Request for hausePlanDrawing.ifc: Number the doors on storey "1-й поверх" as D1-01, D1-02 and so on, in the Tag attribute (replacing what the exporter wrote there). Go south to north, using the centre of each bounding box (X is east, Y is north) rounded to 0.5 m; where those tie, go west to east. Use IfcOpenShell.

First a look at what the model holds.

```python
import ifcopenshell
import ifcopenshell.util.element
import ifcopenshell.util.placement

model = ifcopenshell.open("hausePlanDrawing.ifc")
print(model.schema)
storey = next(s for s in model.by_type("IfcBuildingStorey") if s.Name == "1-й поверх")
doors = [e for e in ifcopenshell.util.element.get_decomposition(storey) if e.is_a("IfcDoor")]
for e in sorted(doors, key=lambda e: e.id()):
    origin = ifcopenshell.util.placement.get_local_placement(e.ObjectPlacement)[:3, 3]
    print(e.id(), e.Tag, e.Name, origin.round(2) + 0.0, sep=" | ")
```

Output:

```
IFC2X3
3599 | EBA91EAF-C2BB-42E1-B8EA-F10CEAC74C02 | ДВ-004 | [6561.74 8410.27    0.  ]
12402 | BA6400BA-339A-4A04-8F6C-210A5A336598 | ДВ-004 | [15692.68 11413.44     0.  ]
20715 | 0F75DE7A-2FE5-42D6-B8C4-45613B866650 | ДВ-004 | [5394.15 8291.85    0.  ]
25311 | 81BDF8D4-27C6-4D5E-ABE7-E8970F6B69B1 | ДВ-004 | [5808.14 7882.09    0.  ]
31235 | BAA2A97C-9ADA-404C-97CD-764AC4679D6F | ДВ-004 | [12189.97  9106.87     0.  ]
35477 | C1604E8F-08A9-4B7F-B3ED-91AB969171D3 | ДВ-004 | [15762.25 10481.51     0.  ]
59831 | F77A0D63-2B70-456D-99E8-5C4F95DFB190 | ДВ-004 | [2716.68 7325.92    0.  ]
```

```python
import ifcopenshell
import ifcopenshell.geom
import ifcopenshell.util.element
import ifcopenshell.util.shape

model = ifcopenshell.open("hausePlanDrawing.ifc")
settings = ifcopenshell.geom.settings()
settings.set("use-world-coords", True)


def centre(element):
    shape = ifcopenshell.geom.create_shape(settings, element)
    return ifcopenshell.util.shape.get_bbox_centroid(shape.geometry)


storey = next(s for s in model.by_type("IfcBuildingStorey") if s.Name == "1-й поверх")
doors = [e for e in ifcopenshell.util.element.get_decomposition(storey) if e.is_a("IfcDoor")]

# Insertion points can sit at a corner or the storey origin, so sort by the geometry (in metres).
centres = {e: centre(e) for e in doors}
doors.sort(key=lambda e: (round(centres[e][1] / 0.5), centres[e][0]))

for i, e in enumerate(doors, start=1):
    number = f"D1-{i:02d}"
    e.Tag = number
    print(e.id(), number)

model.write("hausePlanDrawing_updated.ifc")
```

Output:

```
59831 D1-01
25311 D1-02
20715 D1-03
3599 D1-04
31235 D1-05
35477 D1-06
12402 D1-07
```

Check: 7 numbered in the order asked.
